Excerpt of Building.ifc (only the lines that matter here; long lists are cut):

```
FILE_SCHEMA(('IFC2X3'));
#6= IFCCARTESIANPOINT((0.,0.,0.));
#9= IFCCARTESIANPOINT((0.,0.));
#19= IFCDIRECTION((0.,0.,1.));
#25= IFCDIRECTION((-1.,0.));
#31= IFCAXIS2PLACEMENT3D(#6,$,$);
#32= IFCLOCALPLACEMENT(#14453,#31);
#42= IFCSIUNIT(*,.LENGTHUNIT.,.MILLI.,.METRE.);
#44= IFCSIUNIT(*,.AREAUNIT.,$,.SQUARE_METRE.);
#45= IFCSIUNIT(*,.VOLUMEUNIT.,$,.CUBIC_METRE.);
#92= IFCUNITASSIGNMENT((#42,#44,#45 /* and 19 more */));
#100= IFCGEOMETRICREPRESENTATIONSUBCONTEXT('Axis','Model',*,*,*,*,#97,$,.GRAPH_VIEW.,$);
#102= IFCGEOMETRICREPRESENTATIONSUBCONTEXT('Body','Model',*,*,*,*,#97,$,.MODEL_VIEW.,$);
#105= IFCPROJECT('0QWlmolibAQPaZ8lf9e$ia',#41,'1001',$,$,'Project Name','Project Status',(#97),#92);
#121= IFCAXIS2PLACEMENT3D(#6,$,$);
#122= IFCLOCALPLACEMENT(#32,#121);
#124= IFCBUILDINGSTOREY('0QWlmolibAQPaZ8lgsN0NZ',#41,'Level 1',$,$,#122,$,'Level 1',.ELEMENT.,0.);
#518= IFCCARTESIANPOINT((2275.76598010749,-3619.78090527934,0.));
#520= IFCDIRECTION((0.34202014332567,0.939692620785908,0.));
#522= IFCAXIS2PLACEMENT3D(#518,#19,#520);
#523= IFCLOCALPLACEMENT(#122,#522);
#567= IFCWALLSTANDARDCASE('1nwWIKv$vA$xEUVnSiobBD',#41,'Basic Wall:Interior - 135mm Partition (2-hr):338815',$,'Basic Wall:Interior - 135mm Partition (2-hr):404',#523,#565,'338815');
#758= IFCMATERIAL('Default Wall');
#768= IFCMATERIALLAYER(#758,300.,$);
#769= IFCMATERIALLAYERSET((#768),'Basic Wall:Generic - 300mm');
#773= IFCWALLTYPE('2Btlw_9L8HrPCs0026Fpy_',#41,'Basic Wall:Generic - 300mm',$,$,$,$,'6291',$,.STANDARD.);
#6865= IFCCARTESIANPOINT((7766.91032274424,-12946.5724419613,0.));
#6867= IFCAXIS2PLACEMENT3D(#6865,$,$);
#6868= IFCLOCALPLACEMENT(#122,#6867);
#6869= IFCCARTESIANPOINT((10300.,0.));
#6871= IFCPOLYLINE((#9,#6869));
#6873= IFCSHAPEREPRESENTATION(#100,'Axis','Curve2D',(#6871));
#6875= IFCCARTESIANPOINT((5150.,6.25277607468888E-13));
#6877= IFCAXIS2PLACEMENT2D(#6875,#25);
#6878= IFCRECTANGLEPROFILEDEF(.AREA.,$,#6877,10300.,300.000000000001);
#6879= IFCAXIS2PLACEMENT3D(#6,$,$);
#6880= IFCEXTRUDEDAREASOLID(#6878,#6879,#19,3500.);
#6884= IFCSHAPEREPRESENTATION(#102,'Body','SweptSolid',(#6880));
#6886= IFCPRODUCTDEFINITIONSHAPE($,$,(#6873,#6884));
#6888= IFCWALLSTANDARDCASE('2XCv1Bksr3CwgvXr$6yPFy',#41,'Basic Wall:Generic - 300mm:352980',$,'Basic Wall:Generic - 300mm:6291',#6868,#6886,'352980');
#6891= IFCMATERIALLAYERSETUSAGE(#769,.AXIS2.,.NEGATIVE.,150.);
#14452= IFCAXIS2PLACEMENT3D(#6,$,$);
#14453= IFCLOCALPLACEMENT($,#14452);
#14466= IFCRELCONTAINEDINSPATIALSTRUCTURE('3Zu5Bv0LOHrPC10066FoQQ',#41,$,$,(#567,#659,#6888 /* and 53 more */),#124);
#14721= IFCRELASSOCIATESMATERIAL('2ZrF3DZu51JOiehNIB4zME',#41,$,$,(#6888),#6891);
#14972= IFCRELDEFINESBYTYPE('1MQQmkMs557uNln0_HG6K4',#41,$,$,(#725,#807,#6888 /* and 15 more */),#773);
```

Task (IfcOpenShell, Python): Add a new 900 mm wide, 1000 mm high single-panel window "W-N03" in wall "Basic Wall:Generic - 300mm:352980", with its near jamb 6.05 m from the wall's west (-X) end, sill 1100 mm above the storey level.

```python
import numpy as np
import ifcopenshell
import ifcopenshell.api.feature
import ifcopenshell.api.geometry
import ifcopenshell.api.root
import ifcopenshell.api.spatial
import ifcopenshell.api.type
import ifcopenshell.geom
import ifcopenshell.util.element
import ifcopenshell.util.placement
import ifcopenshell.util.representation
import ifcopenshell.util.shape
import ifcopenshell.util.unit

model = ifcopenshell.open("Building.ifc")
unit_scale = ifcopenshell.util.unit.calculate_unit_scale(model)
settings = ifcopenshell.geom.settings()


def volume(element):
    """Net volume in cubic metres, openings subtracted."""
    shape = ifcopenshell.geom.create_shape(settings, element)
    return ifcopenshell.util.shape.get_volume(shape.geometry)


wall = model.by_id(6888)
storey = ifcopenshell.util.element.get_container(wall, ifc_class="IfcBuildingStorey")
context = ifcopenshell.util.representation.get_context(model, "Model", "Body", "MODEL_VIEW")
before = volume(wall)

width, height, from_end, sill = 0.9, 1, 6.05, 1.1  # metres

# The wall runs along its own X axis, and the end named is its -X end.
wall_shape = ifcopenshell.geom.create_shape(settings, wall)
x, y, z = ifcopenshell.util.shape.get_vertices(wall_shape.geometry).T
start = x.min() + from_end
face, thickness = float(y.min()), float(y.max() - y.min())
wall_matrix = ifcopenshell.util.placement.get_local_placement(wall.ObjectPlacement)
level = ifcopenshell.util.placement.get_local_placement(storey.ObjectPlacement)[2, 3]


def in_wall(x, y):
    """Placement at x, y metres in the wall's axes, at sill height."""
    matrix = wall_matrix.copy()
    matrix[:, 3] = wall_matrix @ np.array([x / unit_scale, y / unit_scale, 0.0, 1.0])
    matrix[2, 3] = level + sill / unit_scale
    return matrix


# Opening: a box that overshoots both wall faces by 50 mm.
opening = ifcopenshell.api.root.create_entity(model, ifc_class="IfcOpeningElement")
box = ifcopenshell.api.geometry.add_wall_representation(
    model, context=context, length=width, height=height, thickness=thickness + 0.1
)
ifcopenshell.api.geometry.assign_representation(model, product=opening, representation=box)
ifcopenshell.api.geometry.edit_object_placement(model, product=opening, matrix=in_wall(start, face - 0.05), is_si=False)
ifcopenshell.api.feature.add_feature(model, feature=opening, element=wall)

window = ifcopenshell.api.root.create_entity(model, ifc_class="IfcWindow", name="W-N03")
window.OverallWidth, window.OverallHeight = width / unit_scale, height / unit_scale
body = ifcopenshell.api.geometry.add_window_representation(
    model,
    context=context,
    overall_width=window.OverallWidth,
    overall_height=window.OverallHeight,
    partition_type="SINGLE_PANEL",
)
ifcopenshell.api.geometry.assign_representation(model, product=window, representation=body)
ifcopenshell.api.spatial.assign_container(model, products=[window], relating_structure=storey)
fills = ifcopenshell.api.feature.add_filling(model, opening=opening, element=window)
fills.OwnerHistory = window.OwnerHistory  # required in IFC2X3

# IFC2X3 keeps the operation on the window style.
style = ifcopenshell.api.root.create_entity(model, ifc_class="IfcWindowStyle", name="W-N03")
style.OperationType, style.ConstructionType = "SINGLE_PANEL", "NOTDEFINED"
style.ParameterTakesPrecedence = style.Sizeable = False
ifcopenshell.api.type.assign_type(model, related_objects=[window], relating_type=style)

# Centre the window in the wall's thickness.
ifcopenshell.api.geometry.edit_object_placement(model, product=window, matrix=in_wall(start, face), is_si=False)
window_shape = ifcopenshell.geom.create_shape(settings, window)
depth = ifcopenshell.util.shape.get_vertices(window_shape.geometry)[:, 1]
offset = face + thickness / 2 - (depth.min() + depth.max()) / 2
ifcopenshell.api.geometry.edit_object_placement(model, product=window, matrix=in_wall(start, offset), is_si=False)

after = volume(wall)

print(f"wall volume {before:.3f} -> {after:.3f} m3")

model.write("Building-out.ifc")
```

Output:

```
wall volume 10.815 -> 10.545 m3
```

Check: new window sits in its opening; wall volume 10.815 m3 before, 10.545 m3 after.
